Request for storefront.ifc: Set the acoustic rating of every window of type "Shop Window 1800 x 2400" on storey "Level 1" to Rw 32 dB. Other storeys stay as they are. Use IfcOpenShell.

First a look at what the model holds.

```python
import ifcopenshell
import ifcopenshell.util.element

model = ifcopenshell.open("storefront.ifc")
print(model.schema)
storey = next(s for s in model.by_type("IfcBuildingStorey") if s.Name == "Level 1")
windows = [e for e in ifcopenshell.util.element.get_decomposition(storey) if e.is_a("IfcWindow")]
seen = {}
for e in windows:
    element_type = ifcopenshell.util.element.get_type(e)
    key = (element_type.Name if element_type != e and element_type else None, ifcopenshell.util.element.get_pset(e, "Pset_WindowCommon", "AcousticRating"))
    seen[key] = seen.get(key, 0) + 1
for (name, value), count in sorted(seen.items(), key=str):
    print(count, "x", name, "|", value)
```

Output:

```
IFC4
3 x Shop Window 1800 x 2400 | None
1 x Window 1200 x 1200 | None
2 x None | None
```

```python
import ifcopenshell
import ifcopenshell.api.pset
import ifcopenshell.util.element

model = ifcopenshell.open("storefront.ifc")

storey = next(s for s in model.by_type("IfcBuildingStorey") if s.Name == "Level 1")
windows = [e for e in ifcopenshell.util.element.get_decomposition(storey) if e.is_a("IfcWindow")]

count = 0
for e in windows:
    element_type = ifcopenshell.util.element.get_type(e)
    if element_type in (None, e) or element_type.Name != "Shop Window 1800 x 2400":
        continue
    # add_pset returns the element's existing set when there is one.
    pset = ifcopenshell.api.pset.add_pset(model, product=e, name="Pset_WindowCommon")
    ifcopenshell.api.pset.edit_pset(model, pset=pset, properties={"AcousticRating": "Rw 32 dB"})
    count += 1

print(count, "windows updated")

model.write("storefront_updated.ifc")
```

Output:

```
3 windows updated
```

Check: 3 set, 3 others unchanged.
